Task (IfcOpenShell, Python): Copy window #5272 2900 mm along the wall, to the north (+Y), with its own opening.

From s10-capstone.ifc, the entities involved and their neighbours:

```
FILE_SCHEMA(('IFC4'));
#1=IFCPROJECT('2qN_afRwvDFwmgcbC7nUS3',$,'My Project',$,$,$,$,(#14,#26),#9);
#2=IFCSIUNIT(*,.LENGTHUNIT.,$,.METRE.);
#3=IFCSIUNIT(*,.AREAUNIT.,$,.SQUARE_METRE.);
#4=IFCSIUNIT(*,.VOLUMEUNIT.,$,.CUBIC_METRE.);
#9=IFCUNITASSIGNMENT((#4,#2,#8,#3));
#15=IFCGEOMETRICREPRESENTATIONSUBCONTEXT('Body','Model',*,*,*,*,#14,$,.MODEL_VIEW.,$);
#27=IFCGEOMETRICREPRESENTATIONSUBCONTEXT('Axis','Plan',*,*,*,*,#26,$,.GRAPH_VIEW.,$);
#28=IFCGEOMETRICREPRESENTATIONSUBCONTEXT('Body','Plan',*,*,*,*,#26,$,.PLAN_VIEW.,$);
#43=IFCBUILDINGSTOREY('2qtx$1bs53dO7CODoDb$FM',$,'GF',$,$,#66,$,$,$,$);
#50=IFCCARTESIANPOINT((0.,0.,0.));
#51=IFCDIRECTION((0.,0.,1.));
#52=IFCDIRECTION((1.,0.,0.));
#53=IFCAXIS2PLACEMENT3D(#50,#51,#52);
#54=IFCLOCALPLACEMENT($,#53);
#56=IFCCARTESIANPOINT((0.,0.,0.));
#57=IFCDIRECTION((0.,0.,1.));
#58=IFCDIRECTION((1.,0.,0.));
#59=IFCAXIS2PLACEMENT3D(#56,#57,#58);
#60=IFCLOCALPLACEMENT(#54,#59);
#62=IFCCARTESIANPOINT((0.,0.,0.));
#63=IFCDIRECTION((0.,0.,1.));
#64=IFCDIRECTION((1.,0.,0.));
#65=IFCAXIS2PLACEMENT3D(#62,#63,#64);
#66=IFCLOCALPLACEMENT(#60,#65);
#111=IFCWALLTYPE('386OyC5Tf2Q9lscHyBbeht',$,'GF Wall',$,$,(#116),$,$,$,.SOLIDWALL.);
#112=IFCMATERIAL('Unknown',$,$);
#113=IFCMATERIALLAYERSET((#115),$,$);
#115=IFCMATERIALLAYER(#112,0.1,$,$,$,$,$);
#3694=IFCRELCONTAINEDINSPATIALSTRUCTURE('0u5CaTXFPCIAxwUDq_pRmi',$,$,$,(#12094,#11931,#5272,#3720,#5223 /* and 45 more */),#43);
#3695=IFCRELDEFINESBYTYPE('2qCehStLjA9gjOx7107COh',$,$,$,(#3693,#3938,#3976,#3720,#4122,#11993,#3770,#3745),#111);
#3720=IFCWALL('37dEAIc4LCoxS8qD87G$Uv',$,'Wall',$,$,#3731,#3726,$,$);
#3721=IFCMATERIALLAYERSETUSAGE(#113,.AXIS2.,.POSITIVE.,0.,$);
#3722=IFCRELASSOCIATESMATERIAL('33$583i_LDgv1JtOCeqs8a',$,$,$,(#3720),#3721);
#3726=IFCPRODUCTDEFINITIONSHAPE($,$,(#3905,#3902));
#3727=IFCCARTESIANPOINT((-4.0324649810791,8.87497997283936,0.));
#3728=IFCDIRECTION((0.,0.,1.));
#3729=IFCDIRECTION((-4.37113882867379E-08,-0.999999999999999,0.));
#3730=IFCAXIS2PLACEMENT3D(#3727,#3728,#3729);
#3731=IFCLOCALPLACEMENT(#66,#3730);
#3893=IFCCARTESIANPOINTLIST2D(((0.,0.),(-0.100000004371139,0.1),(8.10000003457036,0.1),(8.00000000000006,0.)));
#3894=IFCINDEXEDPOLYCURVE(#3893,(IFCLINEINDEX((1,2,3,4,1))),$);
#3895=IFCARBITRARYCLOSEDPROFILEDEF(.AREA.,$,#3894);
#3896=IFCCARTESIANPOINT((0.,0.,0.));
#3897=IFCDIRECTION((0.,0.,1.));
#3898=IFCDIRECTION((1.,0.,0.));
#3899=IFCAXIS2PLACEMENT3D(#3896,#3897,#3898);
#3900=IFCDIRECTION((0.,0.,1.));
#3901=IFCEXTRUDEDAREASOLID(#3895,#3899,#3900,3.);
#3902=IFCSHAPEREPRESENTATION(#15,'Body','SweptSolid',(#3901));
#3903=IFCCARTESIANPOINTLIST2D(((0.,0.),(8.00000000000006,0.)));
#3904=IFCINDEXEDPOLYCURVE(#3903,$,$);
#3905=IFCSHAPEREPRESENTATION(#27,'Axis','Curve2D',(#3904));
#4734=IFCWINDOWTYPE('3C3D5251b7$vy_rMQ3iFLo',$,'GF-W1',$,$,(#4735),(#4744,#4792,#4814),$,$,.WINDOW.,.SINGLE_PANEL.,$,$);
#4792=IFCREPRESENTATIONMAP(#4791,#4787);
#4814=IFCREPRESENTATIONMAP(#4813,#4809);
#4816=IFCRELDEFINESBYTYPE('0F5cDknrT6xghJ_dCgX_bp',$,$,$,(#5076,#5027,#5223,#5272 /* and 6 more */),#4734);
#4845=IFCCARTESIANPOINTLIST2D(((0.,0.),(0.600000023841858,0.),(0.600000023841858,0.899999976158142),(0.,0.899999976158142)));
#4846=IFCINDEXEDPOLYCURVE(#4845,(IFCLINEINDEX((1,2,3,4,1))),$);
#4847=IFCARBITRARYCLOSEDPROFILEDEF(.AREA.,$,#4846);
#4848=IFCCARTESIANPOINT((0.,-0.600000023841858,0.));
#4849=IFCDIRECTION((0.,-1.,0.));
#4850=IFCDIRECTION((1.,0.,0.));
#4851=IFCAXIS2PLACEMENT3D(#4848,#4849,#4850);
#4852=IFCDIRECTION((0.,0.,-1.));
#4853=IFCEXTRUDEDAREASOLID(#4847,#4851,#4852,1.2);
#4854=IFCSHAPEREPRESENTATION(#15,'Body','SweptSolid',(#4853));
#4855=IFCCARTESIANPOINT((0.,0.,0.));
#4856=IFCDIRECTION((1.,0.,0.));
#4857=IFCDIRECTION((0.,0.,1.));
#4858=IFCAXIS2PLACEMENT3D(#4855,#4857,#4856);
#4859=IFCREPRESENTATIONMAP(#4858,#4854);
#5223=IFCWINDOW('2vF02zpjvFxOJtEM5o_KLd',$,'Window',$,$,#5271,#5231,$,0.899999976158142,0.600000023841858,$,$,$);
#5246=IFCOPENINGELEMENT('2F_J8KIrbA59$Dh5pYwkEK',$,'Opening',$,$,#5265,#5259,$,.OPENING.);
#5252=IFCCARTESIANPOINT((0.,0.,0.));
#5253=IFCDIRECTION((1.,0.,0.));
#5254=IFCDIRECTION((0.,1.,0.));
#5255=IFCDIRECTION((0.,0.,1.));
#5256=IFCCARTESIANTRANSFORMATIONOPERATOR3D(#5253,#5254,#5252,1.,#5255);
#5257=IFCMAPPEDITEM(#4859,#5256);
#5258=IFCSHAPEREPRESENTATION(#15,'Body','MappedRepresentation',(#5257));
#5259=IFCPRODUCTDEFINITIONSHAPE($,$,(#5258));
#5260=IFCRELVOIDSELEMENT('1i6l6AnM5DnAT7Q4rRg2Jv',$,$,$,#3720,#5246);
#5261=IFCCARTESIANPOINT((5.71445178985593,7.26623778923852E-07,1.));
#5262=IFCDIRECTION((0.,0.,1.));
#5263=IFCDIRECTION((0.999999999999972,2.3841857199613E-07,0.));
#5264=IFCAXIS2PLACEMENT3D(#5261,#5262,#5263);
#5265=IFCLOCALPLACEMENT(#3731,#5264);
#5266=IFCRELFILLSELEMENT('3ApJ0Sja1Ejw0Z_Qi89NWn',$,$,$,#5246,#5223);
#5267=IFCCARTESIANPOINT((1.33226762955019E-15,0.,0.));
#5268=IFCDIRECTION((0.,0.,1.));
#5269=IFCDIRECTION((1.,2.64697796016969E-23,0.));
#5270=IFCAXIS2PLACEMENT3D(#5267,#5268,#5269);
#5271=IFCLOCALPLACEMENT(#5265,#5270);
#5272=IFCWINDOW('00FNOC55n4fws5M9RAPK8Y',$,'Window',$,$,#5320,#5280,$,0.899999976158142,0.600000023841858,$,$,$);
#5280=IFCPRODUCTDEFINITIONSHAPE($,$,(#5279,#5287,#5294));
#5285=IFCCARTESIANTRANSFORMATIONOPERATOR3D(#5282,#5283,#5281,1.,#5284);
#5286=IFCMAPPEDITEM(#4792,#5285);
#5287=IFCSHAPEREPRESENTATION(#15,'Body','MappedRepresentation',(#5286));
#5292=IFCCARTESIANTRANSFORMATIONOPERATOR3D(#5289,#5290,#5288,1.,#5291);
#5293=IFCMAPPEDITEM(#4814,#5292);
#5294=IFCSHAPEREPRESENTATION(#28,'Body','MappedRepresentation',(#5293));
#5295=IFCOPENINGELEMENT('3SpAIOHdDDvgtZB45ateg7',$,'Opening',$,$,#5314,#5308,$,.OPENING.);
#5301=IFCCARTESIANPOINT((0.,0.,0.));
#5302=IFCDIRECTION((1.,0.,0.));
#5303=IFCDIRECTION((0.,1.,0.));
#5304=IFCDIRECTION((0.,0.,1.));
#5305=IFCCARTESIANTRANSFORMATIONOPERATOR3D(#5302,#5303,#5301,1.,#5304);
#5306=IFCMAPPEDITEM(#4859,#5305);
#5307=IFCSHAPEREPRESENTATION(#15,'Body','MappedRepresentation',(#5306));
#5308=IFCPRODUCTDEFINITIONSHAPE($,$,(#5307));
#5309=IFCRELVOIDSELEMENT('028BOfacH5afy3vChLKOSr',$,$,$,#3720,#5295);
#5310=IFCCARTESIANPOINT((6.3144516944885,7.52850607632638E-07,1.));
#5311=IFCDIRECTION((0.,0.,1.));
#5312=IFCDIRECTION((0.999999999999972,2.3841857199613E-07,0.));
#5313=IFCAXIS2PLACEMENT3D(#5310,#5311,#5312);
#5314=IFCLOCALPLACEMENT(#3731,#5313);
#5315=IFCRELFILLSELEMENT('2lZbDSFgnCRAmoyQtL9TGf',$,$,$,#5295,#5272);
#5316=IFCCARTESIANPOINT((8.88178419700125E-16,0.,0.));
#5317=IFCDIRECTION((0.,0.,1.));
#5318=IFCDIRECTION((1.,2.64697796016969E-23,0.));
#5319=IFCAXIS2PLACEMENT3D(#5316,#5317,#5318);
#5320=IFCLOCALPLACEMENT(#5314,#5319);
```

```python
import ifcopenshell
import ifcopenshell.api.feature
import ifcopenshell.api.geometry
import ifcopenshell.api.root
import ifcopenshell.geom
import ifcopenshell.util.element
import ifcopenshell.util.placement
import ifcopenshell.util.shape
import ifcopenshell.util.unit

model = ifcopenshell.open("s10-capstone.ifc")
unit_scale = ifcopenshell.util.unit.calculate_unit_scale(model)
settings = ifcopenshell.geom.settings()


def volume(element):
    """Net volume in cubic metres, openings subtracted."""
    shape = ifcopenshell.geom.create_shape(settings, element)
    return ifcopenshell.util.shape.get_volume(shape.geometry)


window = model.by_guid("00FNOC55n4fws5M9RAPK8Y")
opening = window.FillsVoids[0].RelatingOpeningElement
wall = opening.VoidsElements[0].RelatingBuildingElement
before = volume(wall)
shift = ifcopenshell.util.placement.get_local_placement(wall.ObjectPlacement)[:3, 0] * -2.9 / unit_scale

# copy_class copies the void relationship, type, container and properties, but no geometry.
new_opening = ifcopenshell.api.root.copy_class(model, product=opening)
new_opening.Representation = ifcopenshell.util.element.copy_deep(
    model, opening.Representation, exclude=["IfcGeometricRepresentationContext", "IfcRepresentationMap"]
)
new_window = ifcopenshell.api.root.copy_class(model, product=window)
new_window.Representation = ifcopenshell.util.element.copy_deep(
    model, window.Representation, exclude=["IfcGeometricRepresentationContext", "IfcRepresentationMap"]
)
ifcopenshell.api.feature.add_filling(model, opening=new_opening, element=new_window)

for old, new in ((opening, new_opening), (window, new_window)):
    matrix = ifcopenshell.util.placement.get_local_placement(old.ObjectPlacement)
    matrix[:3, 3] += shift
    ifcopenshell.api.geometry.edit_object_placement(model, product=new, matrix=matrix, is_si=False)

after = volume(wall)

print(f"wall volume {before:.3f} -> {after:.3f} m3")

model.write("s10-capstone_updated.ifc")
```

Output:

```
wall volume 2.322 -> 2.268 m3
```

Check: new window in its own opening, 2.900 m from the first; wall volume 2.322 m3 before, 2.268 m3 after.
